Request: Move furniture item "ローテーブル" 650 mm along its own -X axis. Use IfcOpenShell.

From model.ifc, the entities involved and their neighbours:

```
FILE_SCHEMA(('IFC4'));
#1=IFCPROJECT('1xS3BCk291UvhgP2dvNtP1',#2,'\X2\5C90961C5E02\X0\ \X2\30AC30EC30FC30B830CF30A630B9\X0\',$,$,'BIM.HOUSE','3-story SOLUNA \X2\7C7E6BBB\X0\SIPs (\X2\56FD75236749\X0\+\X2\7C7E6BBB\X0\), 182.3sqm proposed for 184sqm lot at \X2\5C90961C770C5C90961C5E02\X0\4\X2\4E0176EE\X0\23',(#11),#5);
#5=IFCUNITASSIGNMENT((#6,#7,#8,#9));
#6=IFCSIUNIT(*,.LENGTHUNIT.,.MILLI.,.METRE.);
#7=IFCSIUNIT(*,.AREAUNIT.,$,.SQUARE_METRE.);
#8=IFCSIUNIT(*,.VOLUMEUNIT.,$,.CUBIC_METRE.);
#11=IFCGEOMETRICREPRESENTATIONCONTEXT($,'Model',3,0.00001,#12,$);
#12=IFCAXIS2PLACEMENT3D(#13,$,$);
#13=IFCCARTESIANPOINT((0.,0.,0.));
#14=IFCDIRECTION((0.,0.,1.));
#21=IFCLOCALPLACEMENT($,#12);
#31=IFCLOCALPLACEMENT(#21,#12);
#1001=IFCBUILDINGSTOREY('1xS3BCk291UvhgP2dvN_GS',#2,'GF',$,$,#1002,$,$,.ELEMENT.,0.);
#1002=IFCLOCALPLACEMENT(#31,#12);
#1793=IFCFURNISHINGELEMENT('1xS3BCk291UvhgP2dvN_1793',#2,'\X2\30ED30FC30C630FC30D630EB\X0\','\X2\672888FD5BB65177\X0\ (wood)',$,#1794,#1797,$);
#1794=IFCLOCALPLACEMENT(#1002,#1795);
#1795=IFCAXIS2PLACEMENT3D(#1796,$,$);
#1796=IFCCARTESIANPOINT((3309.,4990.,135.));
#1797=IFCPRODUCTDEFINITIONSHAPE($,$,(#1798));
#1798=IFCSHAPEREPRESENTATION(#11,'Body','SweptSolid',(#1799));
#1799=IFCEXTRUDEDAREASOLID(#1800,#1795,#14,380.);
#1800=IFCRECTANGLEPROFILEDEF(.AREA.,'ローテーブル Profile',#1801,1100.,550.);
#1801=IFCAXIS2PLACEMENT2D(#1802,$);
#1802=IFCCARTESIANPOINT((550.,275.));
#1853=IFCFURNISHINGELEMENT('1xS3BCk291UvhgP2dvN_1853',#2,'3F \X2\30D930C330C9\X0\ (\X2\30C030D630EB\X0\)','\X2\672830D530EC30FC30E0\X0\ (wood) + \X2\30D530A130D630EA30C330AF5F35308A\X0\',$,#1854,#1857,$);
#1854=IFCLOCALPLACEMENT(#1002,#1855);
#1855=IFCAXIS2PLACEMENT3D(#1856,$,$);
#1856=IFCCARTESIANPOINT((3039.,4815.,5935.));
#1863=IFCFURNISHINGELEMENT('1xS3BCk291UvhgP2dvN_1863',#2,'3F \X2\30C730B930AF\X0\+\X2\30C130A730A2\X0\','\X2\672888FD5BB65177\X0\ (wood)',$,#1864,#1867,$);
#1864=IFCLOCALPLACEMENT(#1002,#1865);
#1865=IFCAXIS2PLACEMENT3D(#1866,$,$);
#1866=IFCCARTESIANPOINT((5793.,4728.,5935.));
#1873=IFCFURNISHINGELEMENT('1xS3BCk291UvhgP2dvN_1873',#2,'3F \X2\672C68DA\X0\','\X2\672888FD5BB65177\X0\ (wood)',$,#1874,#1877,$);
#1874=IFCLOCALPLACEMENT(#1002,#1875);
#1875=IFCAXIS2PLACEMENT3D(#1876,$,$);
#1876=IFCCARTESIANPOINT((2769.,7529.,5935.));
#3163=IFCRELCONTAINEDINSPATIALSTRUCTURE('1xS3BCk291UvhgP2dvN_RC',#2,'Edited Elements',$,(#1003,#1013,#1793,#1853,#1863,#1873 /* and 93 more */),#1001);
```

```python
import ifcopenshell
import ifcopenshell.api.geometry
import ifcopenshell.util.placement

model = ifcopenshell.open("model.ifc")

item = model.by_guid("1xS3BCk291UvhgP2dvN_1793")
matrix = ifcopenshell.util.placement.get_local_placement(item.ObjectPlacement)
matrix[:3, 3] -= matrix[:3, 0] * 650.0
ifcopenshell.api.geometry.edit_object_placement(model, product=item, matrix=matrix, is_si=False)

print(ifcopenshell.util.placement.get_local_placement(item.ObjectPlacement).round(3) + 0.0)

model.write("model-out.ifc")
```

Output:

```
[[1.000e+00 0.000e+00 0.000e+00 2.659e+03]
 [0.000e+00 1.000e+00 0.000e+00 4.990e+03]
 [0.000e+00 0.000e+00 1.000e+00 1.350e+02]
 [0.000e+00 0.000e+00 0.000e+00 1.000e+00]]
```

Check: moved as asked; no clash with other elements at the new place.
